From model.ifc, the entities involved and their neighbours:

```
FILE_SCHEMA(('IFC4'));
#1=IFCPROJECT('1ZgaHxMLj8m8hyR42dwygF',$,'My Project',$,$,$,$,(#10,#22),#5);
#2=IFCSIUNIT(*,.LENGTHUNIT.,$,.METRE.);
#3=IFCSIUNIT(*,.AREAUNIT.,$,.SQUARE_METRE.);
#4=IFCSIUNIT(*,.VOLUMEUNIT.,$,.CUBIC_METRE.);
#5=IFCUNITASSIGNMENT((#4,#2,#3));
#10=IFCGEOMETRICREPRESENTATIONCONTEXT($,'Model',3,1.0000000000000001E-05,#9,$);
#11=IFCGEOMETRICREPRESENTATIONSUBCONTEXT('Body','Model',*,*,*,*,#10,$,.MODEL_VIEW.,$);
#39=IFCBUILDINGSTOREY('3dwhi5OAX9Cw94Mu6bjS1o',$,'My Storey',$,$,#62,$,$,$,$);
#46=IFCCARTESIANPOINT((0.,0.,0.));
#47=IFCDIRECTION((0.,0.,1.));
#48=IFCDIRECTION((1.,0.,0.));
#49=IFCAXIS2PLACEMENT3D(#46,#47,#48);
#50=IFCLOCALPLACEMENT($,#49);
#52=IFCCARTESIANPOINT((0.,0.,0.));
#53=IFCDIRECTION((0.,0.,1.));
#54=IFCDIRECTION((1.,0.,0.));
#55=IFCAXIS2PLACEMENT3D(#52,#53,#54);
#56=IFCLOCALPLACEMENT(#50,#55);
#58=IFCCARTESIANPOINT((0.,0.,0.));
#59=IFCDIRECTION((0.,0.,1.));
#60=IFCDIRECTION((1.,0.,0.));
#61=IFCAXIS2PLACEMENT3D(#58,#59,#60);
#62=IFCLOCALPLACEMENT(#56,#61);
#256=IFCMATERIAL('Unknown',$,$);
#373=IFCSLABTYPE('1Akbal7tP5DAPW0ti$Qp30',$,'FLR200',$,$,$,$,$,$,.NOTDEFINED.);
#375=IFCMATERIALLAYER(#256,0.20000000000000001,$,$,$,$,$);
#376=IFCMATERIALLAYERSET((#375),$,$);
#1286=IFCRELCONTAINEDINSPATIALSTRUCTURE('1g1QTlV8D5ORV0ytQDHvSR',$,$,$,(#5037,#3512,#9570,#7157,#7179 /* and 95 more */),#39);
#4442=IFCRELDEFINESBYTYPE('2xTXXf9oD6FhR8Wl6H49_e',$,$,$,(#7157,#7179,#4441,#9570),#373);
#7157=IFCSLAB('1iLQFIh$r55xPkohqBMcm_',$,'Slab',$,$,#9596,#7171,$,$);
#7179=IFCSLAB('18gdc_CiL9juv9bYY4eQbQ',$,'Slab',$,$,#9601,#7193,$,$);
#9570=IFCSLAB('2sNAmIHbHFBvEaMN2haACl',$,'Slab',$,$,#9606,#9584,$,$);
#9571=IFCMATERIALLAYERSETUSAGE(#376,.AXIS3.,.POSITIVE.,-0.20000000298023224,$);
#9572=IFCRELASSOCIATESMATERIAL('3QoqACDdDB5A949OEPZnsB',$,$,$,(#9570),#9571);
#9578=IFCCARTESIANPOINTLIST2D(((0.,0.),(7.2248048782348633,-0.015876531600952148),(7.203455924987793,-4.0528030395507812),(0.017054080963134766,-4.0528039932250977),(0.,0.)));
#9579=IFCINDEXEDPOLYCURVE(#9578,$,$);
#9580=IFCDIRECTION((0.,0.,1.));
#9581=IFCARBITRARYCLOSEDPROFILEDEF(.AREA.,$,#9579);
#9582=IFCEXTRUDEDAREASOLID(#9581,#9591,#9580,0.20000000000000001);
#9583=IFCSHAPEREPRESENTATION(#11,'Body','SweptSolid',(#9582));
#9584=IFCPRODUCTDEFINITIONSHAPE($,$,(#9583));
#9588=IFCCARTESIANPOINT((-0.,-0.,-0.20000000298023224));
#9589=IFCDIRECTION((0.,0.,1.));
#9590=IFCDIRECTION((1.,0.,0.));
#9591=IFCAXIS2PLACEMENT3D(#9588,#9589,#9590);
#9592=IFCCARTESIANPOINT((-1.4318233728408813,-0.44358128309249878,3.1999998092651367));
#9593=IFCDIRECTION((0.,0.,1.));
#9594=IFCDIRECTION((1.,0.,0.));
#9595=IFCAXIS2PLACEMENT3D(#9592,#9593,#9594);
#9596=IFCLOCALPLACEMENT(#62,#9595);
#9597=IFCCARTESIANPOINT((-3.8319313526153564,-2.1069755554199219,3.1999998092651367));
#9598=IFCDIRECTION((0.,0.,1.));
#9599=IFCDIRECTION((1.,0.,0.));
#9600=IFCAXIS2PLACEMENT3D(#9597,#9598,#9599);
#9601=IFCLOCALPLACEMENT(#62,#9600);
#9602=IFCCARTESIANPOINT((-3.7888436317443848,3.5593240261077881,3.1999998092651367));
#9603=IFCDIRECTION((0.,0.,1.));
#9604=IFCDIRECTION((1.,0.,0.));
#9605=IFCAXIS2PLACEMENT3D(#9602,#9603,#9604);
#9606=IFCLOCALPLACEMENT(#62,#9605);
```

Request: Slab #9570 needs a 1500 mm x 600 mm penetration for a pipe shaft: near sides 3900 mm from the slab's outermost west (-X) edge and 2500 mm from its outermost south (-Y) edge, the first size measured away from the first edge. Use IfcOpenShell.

```python
import numpy as np
import ifcopenshell
import ifcopenshell.api.feature
import ifcopenshell.api.geometry
import ifcopenshell.api.root
import ifcopenshell.geom
import ifcopenshell.util.placement
import ifcopenshell.util.representation
import ifcopenshell.util.shape
import ifcopenshell.util.unit

model = ifcopenshell.open("model.ifc")
unit_scale = ifcopenshell.util.unit.calculate_unit_scale(model)
settings = ifcopenshell.geom.settings()


def volume(element):
    """Net volume in cubic metres, openings subtracted."""
    shape = ifcopenshell.geom.create_shape(settings, element)
    return ifcopenshell.util.shape.get_volume(shape.geometry)


slab = model.by_id(9570)
before = volume(slab)

# Extent in the slab's own axes, in metres. The edges named are its -X and -Y sides.
slab_shape = ifcopenshell.geom.create_shape(settings, slab)
vertices = ifcopenshell.util.shape.get_vertices(slab_shape.geometry)
x_min, y_min, bottom = vertices.min(axis=0)
top = vertices[:, 2].max()

opening = ifcopenshell.api.root.create_entity(model, ifc_class="IfcOpeningElement", name="Pipe shaft opening", predefined_type="OPENING")
context = ifcopenshell.util.representation.get_context(model, "Model", "Body", "MODEL_VIEW")
width, depth = 1.5, 0.6
outline = [(0.0, 0.0), (width, 0.0), (width, depth), (0.0, depth), (0.0, 0.0)]
# Overshoot both faces by 50 mm so the cut is clean.
shape = ifcopenshell.api.geometry.add_slab_representation(
    model, context=context, depth=top - bottom + 0.1, polyline=outline
)
ifcopenshell.api.geometry.assign_representation(model, product=opening, representation=shape)

matrix = ifcopenshell.util.placement.get_local_placement(slab.ObjectPlacement)
matrix[:, 3] = matrix @ np.append(np.array([x_min + 3.9, y_min + 2.5, bottom - 0.05]) / unit_scale, 1.0)
ifcopenshell.api.geometry.edit_object_placement(model, product=opening, matrix=matrix, is_si=False)
ifcopenshell.api.feature.add_feature(model, feature=opening, element=slab)

after = volume(slab)

print(f"slab volume {before:.3f} -> {after:.3f} m3")

model.write("model_v2.ifc")
```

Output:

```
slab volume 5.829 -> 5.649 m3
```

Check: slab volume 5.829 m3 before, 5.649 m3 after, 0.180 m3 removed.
